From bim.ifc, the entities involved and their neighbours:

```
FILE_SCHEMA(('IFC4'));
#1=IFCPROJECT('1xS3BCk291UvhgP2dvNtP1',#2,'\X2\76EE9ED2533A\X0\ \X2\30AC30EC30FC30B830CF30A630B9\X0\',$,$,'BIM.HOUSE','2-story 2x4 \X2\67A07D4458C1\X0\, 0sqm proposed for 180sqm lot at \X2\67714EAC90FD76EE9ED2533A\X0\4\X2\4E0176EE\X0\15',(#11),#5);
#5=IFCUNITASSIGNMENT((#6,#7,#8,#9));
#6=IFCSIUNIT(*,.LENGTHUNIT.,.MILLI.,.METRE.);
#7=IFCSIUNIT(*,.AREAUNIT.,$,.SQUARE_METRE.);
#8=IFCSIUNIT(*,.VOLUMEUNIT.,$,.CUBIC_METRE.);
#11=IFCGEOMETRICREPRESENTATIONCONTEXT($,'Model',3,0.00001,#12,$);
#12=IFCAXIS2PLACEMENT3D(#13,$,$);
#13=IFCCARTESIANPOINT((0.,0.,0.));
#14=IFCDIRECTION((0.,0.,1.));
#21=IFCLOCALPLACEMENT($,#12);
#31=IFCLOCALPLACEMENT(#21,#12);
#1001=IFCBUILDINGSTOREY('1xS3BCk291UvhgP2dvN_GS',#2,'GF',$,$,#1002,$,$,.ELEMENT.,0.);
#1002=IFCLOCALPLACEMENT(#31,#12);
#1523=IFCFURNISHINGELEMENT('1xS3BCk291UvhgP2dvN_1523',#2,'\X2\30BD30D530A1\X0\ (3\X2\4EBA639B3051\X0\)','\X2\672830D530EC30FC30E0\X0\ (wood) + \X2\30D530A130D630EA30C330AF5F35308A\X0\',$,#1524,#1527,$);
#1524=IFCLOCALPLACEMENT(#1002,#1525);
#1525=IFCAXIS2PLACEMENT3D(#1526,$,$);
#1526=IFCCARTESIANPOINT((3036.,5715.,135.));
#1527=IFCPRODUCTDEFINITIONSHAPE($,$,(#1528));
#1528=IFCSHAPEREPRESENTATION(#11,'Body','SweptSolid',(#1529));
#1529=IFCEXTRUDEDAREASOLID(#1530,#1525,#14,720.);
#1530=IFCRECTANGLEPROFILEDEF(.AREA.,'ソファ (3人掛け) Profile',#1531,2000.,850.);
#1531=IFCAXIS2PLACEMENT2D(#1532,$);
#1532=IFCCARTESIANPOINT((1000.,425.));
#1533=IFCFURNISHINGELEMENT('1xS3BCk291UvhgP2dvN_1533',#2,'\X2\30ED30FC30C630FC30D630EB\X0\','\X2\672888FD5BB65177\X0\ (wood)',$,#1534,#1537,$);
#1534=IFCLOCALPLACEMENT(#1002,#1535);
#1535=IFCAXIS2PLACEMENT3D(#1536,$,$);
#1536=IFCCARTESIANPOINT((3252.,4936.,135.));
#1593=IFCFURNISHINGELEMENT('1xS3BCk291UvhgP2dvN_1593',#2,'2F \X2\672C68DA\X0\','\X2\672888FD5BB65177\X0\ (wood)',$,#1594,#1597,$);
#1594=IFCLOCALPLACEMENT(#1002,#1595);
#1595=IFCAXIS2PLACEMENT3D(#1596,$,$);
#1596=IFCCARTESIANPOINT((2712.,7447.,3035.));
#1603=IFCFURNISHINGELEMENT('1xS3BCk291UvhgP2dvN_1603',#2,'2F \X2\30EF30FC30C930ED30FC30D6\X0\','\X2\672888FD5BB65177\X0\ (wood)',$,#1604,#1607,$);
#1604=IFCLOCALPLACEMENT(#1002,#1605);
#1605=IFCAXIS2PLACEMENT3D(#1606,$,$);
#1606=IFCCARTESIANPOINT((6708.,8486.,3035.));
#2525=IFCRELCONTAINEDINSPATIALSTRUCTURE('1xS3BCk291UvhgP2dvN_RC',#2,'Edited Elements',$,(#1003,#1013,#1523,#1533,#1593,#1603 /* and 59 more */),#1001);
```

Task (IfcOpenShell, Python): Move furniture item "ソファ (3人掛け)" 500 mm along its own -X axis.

```python
import ifcopenshell
import ifcopenshell.api.geometry
import ifcopenshell.util.placement

model = ifcopenshell.open("bim.ifc")

item = model.by_guid("1xS3BCk291UvhgP2dvN_1523")
matrix = ifcopenshell.util.placement.get_local_placement(item.ObjectPlacement)
matrix[:3, 3] -= matrix[:3, 0] * 500.0
ifcopenshell.api.geometry.edit_object_placement(model, product=item, matrix=matrix, is_si=False)

print(ifcopenshell.util.placement.get_local_placement(item.ObjectPlacement).round(3) + 0.0)

model.write("bim_updated.ifc")
```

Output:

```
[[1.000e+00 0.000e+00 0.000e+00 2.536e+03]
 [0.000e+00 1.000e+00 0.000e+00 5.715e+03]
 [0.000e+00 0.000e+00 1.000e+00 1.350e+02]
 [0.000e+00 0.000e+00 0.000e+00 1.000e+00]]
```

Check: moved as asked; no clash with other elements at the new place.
